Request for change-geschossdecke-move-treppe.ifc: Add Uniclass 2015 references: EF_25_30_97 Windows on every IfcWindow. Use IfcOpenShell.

First a look at what the model holds.

```python
import ifcopenshell

model = ifcopenshell.open("change-geschossdecke-move-treppe.ifc")
print(model.schema)
print("classifications:", [c.Name for c in model.by_type("IfcClassification")])
for ifc_class in ("IfcDoor", "IfcRoof", "IfcStair", "IfcWall", "IfcWindow"):
    print(ifc_class, len(model.by_type(ifc_class)))
```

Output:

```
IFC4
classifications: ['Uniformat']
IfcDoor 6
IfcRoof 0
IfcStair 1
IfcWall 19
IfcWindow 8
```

```python
import ifcopenshell
import ifcopenshell.api.classification

model = ifcopenshell.open("change-geschossdecke-move-treppe.ifc")

system = ifcopenshell.api.classification.add_classification(model, classification="Uniclass 2015")

codes = {
    "IfcWindow": ("EF_25_30_97", "Windows"),
}
for ifc_class, (code, name) in codes.items():
    products = model.by_type(ifc_class)
    ifcopenshell.api.classification.add_reference(
        model, products=products, classification=system, identification=code, name=name
    )
    print(code, len(products))

model.write("change-geschossdecke-move-treppe_edited.ifc")
```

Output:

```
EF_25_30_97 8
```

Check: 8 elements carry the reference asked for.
